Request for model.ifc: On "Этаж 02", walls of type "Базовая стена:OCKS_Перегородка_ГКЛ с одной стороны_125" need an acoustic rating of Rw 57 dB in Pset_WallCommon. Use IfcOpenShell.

First a look at what the model holds.

```python
import ifcopenshell
import ifcopenshell.util.element

model = ifcopenshell.open("model.ifc")
print(model.schema)
storey = next(s for s in model.by_type("IfcBuildingStorey") if s.Name == "Этаж 02")
walls = [e for e in ifcopenshell.util.element.get_decomposition(storey) if e.is_a("IfcWall")]
seen = {}
for e in walls:
    element_type = ifcopenshell.util.element.get_type(e)
    key = (element_type.Name if element_type != e and element_type else None, ifcopenshell.util.element.get_pset(e, "Pset_WallCommon", "AcousticRating"))
    seen[key] = seen.get(key, 0) + 1
for (name, value), count in sorted(seen.items(), key=str):
    print(count, "x", name, "|", value)
```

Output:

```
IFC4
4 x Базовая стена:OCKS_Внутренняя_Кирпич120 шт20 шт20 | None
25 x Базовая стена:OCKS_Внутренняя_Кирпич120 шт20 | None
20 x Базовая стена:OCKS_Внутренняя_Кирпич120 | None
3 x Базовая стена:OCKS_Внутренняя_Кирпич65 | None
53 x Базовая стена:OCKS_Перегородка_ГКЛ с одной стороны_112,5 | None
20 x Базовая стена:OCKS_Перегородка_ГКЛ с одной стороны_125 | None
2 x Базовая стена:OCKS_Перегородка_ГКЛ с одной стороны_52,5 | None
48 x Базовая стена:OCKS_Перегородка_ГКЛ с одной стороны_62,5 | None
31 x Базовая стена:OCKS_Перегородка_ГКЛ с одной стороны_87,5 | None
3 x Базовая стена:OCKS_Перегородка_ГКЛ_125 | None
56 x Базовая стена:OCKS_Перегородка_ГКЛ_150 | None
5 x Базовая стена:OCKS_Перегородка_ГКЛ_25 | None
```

```python
import ifcopenshell
import ifcopenshell.api.pset
import ifcopenshell.util.element

model = ifcopenshell.open("model.ifc")

storey = next(s for s in model.by_type("IfcBuildingStorey") if s.Name == "Этаж 02")
walls = [e for e in ifcopenshell.util.element.get_decomposition(storey) if e.is_a("IfcWall")]

count = 0
for e in walls:
    element_type = ifcopenshell.util.element.get_type(e)
    if element_type in (None, e) or element_type.Name != "Базовая стена:OCKS_Перегородка_ГКЛ с одной стороны_125":
        continue
    # add_pset returns the element's existing set when there is one.
    pset = ifcopenshell.api.pset.add_pset(model, product=e, name="Pset_WallCommon")
    ifcopenshell.api.pset.edit_pset(model, pset=pset, properties={"AcousticRating": "Rw 57 dB"})
    count += 1

print(count, "walls updated")

model.write("model_rev.ifc")
```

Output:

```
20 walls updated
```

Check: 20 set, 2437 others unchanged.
